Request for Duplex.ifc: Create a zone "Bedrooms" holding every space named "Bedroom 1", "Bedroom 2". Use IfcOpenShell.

First a look at what the model holds.

```python
import ifcopenshell

model = ifcopenshell.open("Duplex.ifc")
print(model.schema)
seen = {}
for space in model.by_type("IfcSpace"):
    seen[space.LongName] = seen.get(space.LongName, 0) + 1
for name, count in sorted(seen.items(), key=str):
    print(count, "x", name)
print("zones:", [z.Name for z in model.by_type("IfcZone")][:20])
```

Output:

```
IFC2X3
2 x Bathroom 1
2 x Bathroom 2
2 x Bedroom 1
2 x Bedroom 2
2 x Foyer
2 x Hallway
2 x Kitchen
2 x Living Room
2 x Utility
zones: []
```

```python
import ifcopenshell
import ifcopenshell.api.group
import ifcopenshell.api.root

model = ifcopenshell.open("Duplex.ifc")

names = {"Bedroom 1", "Bedroom 2"}
spaces = [s for s in model.by_type("IfcSpace") if s.LongName in names]

zone = ifcopenshell.api.root.create_entity(model, ifc_class="IfcZone", name="Bedrooms")
ifcopenshell.api.group.assign_group(model, products=spaces, group=zone)
print(len(spaces), "spaces in", zone.Name)

model.write("Duplex_edited.ifc")
```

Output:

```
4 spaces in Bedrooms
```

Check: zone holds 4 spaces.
